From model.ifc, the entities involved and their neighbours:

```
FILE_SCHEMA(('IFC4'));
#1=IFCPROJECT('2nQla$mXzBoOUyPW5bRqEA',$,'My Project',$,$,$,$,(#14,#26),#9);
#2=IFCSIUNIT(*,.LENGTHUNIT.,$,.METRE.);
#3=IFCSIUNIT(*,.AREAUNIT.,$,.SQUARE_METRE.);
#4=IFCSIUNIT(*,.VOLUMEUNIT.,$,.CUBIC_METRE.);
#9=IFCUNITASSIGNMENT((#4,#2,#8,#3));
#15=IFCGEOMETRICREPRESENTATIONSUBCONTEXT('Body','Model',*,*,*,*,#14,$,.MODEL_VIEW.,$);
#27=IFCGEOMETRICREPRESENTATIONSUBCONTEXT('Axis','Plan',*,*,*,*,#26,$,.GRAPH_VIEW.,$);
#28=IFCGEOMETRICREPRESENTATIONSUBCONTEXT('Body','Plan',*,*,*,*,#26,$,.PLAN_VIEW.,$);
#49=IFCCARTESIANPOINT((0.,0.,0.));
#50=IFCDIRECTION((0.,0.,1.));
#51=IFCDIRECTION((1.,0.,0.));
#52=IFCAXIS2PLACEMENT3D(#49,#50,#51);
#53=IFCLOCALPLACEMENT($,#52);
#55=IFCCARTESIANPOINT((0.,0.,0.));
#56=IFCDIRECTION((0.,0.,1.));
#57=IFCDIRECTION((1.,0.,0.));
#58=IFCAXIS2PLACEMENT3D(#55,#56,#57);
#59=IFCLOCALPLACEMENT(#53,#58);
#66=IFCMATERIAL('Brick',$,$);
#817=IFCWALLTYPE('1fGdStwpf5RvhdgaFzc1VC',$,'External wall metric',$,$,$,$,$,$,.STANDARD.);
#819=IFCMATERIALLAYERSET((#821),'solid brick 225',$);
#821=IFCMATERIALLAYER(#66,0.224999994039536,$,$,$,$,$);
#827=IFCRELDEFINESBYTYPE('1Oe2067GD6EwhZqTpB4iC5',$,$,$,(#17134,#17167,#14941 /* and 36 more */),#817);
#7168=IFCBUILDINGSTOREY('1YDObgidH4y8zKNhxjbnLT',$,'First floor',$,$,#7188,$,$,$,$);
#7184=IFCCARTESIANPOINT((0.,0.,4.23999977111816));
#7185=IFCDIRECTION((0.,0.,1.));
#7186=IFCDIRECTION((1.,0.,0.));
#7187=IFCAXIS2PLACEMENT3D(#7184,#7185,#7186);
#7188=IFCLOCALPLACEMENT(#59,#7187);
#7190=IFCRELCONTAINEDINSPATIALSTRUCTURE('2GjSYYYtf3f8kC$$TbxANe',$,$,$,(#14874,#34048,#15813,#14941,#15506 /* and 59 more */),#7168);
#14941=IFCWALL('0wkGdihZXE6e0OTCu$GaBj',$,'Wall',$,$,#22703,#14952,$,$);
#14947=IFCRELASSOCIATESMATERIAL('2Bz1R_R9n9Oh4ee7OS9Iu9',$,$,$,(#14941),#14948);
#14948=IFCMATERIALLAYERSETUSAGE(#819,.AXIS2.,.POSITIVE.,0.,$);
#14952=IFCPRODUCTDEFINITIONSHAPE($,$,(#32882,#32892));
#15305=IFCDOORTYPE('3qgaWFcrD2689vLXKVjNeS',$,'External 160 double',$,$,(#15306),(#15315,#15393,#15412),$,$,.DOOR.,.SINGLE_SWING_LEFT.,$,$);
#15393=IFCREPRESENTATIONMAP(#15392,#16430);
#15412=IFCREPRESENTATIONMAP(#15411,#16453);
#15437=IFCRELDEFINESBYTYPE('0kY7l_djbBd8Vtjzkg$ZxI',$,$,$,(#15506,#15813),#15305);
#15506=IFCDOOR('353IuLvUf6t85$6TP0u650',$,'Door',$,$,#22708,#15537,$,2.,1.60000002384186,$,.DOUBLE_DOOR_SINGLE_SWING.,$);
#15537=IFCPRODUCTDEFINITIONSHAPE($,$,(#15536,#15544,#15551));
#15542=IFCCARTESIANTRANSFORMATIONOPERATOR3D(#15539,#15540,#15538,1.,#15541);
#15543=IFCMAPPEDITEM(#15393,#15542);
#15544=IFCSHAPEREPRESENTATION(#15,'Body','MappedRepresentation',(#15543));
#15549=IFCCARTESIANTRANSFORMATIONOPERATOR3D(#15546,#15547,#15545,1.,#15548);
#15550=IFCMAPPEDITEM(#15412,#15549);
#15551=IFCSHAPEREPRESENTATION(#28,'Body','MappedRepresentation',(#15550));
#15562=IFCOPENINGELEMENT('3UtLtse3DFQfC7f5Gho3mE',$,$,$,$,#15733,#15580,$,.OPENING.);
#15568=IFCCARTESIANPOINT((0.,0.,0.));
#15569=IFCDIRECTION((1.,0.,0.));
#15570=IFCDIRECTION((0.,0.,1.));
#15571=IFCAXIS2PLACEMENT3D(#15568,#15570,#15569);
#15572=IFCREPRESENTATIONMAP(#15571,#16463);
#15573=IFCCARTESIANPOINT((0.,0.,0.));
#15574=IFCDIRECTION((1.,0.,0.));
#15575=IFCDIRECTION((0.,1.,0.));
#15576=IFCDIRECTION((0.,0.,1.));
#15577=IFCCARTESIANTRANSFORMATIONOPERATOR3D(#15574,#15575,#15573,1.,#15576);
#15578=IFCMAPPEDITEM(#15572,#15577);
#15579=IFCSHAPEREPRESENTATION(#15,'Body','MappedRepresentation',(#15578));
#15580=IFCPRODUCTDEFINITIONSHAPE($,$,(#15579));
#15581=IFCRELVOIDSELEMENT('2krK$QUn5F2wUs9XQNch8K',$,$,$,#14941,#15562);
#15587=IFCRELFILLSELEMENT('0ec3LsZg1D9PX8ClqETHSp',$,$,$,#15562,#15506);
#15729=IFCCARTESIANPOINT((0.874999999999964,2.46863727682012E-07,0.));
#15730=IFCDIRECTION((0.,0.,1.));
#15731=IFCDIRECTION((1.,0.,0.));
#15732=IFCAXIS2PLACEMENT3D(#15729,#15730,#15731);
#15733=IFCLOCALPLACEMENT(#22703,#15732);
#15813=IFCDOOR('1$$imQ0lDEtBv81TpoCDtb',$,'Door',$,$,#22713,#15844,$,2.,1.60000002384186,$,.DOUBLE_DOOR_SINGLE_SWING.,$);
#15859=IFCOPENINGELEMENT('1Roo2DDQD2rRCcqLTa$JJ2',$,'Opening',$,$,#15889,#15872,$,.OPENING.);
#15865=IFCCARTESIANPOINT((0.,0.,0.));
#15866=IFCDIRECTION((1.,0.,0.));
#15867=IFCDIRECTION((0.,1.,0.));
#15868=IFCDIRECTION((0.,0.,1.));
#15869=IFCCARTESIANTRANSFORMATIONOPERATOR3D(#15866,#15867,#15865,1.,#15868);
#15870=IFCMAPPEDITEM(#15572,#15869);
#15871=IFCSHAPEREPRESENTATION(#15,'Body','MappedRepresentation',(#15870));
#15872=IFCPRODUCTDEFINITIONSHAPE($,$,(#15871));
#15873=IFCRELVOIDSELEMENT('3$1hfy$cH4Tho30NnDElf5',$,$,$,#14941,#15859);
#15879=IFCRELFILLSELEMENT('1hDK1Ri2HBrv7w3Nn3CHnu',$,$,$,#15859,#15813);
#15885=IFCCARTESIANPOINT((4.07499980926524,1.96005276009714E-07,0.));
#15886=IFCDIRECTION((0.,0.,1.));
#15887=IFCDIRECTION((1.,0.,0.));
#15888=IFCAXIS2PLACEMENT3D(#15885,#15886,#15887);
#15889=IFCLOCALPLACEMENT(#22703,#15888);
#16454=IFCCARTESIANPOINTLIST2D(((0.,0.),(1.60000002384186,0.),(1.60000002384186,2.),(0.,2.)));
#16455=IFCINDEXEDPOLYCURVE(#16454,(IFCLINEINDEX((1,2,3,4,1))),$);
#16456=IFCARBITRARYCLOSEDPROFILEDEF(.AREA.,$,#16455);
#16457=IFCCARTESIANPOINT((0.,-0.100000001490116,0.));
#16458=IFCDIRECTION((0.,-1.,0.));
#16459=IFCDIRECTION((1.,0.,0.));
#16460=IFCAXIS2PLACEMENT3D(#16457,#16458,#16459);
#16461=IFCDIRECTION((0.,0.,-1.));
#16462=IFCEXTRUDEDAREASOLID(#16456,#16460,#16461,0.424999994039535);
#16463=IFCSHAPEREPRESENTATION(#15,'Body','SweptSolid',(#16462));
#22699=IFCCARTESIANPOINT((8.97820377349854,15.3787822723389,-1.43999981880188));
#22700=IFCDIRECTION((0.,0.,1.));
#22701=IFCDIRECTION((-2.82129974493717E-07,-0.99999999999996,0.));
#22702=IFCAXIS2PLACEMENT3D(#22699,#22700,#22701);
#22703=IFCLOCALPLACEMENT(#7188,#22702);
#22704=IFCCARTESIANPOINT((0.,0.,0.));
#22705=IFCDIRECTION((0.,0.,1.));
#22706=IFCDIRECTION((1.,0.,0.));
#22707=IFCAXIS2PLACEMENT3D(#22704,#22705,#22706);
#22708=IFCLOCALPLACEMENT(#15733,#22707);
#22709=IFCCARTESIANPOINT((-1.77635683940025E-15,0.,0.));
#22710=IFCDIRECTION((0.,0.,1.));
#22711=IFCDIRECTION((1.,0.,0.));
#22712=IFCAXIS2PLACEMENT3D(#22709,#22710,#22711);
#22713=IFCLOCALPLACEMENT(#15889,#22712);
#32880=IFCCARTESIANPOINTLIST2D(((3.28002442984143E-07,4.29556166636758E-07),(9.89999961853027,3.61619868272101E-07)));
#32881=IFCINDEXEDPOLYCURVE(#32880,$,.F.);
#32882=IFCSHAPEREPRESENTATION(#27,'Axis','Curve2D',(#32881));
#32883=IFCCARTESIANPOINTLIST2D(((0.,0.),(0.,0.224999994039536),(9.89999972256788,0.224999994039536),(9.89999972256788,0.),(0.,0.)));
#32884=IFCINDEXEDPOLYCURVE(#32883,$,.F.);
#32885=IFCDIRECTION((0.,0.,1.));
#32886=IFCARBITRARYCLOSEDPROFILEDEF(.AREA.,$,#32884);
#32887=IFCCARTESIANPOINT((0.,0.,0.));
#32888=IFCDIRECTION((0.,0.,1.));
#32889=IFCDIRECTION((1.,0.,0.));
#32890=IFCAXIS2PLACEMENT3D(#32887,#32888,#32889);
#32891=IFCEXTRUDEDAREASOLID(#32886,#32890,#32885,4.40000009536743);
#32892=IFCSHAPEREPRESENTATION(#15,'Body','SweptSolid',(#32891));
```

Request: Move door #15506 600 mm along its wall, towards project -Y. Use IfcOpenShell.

```python
import ifcopenshell
import ifcopenshell.api.geometry
import ifcopenshell.util.placement

model = ifcopenshell.open("model.ifc")

door = model.by_id(15506)
opening = door.FillsVoids[0].RelatingOpeningElement
wall = opening.VoidsElements[0].RelatingBuildingElement

wall_matrix = ifcopenshell.util.placement.get_local_placement(wall.ObjectPlacement)
shift = wall_matrix[:3, 0] * 0.6
before = ifcopenshell.util.placement.get_local_placement(door.ObjectPlacement)[:3, 3].copy()

# The door is placed relative to its opening, so it follows when the opening moves.
matrix = ifcopenshell.util.placement.get_local_placement(opening.ObjectPlacement)
matrix[:3, 3] += shift
ifcopenshell.api.geometry.edit_object_placement(
    model, product=opening, matrix=matrix, is_si=False, should_transform_children=True
)

after = ifcopenshell.util.placement.get_local_placement(door.ObjectPlacement)[:3, 3]
print("door moved by", (after - before).round(3) + 0.0)

model.write("model_rev.ifc")
```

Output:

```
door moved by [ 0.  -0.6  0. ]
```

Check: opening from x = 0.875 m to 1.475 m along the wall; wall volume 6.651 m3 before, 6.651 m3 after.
